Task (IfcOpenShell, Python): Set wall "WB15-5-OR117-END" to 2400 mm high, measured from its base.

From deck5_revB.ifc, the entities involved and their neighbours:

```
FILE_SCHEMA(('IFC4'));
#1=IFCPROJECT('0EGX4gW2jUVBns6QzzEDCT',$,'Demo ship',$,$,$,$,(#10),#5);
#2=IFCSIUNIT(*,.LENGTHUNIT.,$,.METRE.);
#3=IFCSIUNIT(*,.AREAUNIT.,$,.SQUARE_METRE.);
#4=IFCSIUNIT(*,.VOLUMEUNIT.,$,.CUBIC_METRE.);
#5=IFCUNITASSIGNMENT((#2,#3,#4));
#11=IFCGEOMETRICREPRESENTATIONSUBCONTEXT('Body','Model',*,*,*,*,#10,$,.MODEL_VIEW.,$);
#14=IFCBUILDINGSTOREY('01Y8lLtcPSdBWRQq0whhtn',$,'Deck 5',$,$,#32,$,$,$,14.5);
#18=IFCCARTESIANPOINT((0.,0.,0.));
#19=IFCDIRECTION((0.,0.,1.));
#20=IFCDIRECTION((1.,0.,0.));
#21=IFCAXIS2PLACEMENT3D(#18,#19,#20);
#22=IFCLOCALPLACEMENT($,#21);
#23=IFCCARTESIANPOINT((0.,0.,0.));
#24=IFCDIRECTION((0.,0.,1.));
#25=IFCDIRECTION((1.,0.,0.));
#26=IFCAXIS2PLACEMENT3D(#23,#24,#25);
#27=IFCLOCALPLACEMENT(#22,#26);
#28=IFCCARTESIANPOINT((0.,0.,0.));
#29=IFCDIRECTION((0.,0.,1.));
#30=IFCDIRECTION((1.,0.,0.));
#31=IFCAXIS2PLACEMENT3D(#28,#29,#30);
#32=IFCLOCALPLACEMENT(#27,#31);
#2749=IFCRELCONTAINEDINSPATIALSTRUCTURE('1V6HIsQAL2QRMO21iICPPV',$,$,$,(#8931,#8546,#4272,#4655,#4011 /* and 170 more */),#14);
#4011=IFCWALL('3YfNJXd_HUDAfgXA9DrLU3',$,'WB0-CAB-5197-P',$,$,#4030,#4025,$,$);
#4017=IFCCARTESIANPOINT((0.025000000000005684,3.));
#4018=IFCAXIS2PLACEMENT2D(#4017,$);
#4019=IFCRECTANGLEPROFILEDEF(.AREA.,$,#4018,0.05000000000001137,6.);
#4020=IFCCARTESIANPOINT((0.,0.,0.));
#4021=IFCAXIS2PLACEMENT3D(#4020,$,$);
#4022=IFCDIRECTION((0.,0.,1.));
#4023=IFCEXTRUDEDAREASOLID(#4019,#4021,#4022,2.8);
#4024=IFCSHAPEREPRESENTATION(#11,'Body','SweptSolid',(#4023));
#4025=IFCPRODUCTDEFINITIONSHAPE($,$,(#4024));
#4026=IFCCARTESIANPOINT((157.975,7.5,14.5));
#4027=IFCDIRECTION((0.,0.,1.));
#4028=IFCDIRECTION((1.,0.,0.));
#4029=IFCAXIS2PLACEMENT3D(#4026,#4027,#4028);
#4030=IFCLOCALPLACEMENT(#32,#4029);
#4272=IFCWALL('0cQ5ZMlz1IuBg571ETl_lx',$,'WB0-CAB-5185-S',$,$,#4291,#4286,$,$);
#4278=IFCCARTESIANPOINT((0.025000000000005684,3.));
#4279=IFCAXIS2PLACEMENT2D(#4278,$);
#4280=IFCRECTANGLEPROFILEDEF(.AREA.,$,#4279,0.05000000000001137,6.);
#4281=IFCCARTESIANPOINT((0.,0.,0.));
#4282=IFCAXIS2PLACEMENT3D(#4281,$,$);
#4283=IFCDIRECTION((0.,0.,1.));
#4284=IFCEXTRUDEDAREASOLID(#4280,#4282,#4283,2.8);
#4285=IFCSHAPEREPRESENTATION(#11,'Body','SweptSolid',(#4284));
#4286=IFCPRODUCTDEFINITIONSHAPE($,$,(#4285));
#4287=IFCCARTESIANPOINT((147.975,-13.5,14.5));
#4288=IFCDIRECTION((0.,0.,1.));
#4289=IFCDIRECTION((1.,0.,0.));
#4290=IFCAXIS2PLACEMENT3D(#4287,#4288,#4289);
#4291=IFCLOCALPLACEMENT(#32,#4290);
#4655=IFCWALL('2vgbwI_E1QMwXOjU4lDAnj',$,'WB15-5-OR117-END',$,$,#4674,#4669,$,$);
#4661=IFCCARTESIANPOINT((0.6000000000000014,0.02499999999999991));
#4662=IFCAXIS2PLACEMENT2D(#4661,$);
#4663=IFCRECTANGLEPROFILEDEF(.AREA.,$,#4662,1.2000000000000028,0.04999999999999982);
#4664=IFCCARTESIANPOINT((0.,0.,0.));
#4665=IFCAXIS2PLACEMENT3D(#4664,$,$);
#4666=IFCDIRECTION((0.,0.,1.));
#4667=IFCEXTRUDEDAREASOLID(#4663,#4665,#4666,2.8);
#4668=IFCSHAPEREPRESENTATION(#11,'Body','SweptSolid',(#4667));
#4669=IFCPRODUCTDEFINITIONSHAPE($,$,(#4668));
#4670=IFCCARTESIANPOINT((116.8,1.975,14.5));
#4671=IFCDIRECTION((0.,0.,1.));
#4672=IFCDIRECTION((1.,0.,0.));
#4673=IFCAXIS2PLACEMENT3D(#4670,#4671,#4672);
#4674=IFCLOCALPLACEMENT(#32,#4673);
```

```python
import ifcopenshell
import ifcopenshell.geom
import ifcopenshell.util.representation
import ifcopenshell.util.shape
import ifcopenshell.util.unit

model = ifcopenshell.open("deck5_revB.ifc")
unit_scale = ifcopenshell.util.unit.calculate_unit_scale(model)
settings = ifcopenshell.geom.settings()


def volume(element):
    """Net volume in cubic metres, openings subtracted."""
    shape = ifcopenshell.geom.create_shape(settings, element)
    return ifcopenshell.util.shape.get_volume(shape.geometry)


wall = model.by_guid("2vgbwI_E1QMwXOjU4lDAnj")
before = volume(wall)

body = ifcopenshell.util.representation.get_representation(wall, "Model", "Body")
solid = body.Items[0]
old_height = solid.Depth
solid.Depth = 2.4 / unit_scale
after = volume(wall)

print(f"height {old_height:g} -> {solid.Depth:g}, volume {before:.3f} -> {after:.3f} m3")

model.write("deck5_revB-out.ifc")
```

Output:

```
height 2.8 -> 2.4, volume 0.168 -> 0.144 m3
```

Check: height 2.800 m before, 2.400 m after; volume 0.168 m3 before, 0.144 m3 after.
